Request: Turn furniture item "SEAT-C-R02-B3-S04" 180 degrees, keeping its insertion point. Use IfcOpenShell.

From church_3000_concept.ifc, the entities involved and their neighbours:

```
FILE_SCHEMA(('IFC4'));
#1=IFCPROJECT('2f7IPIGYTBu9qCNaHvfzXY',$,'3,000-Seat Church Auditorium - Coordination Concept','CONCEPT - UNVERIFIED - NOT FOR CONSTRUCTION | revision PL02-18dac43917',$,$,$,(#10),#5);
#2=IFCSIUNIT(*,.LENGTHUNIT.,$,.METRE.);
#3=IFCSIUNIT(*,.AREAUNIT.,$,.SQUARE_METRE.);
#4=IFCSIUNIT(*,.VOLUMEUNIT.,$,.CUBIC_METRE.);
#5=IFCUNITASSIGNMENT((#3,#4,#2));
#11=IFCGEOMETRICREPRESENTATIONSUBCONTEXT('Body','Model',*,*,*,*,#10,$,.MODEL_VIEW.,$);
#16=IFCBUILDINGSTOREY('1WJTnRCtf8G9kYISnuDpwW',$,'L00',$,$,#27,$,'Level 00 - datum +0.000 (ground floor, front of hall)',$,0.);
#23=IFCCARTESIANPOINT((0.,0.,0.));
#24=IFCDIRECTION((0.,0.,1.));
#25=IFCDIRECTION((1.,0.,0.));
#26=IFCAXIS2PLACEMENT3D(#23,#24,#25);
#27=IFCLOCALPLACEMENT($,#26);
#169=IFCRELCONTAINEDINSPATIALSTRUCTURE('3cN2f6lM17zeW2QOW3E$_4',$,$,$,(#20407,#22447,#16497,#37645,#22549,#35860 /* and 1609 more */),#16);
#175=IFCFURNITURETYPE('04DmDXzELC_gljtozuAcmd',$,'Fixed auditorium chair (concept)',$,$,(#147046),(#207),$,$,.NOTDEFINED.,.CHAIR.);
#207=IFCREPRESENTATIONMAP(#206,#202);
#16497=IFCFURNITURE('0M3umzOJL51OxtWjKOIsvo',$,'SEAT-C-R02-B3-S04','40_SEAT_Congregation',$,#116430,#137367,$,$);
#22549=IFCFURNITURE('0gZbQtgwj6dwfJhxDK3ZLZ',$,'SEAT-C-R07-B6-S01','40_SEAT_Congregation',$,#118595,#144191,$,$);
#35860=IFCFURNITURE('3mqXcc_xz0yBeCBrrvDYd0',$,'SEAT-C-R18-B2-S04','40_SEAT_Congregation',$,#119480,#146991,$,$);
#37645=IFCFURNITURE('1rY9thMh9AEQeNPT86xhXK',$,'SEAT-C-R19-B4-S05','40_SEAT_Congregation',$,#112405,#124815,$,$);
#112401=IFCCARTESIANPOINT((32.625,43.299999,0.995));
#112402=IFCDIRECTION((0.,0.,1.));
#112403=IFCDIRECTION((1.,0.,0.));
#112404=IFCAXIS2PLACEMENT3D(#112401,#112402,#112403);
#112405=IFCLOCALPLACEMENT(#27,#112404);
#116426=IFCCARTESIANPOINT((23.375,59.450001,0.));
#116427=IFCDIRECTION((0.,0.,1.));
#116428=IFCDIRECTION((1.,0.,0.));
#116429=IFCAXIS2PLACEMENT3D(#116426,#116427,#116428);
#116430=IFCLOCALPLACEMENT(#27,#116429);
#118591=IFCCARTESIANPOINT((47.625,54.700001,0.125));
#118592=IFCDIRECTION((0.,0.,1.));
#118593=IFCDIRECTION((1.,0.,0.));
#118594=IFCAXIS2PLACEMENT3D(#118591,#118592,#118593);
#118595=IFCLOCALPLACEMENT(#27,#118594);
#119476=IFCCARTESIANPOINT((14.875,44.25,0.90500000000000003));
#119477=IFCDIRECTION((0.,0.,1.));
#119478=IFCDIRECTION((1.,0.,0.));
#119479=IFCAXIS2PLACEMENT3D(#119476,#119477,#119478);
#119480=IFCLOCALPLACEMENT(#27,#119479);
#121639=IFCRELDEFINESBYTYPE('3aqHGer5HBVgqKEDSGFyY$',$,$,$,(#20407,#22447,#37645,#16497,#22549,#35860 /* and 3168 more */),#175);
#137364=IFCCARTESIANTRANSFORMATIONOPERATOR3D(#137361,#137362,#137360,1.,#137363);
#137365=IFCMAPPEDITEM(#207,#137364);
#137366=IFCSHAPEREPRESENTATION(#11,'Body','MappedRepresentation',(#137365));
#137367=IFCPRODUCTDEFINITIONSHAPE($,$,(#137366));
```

```python
import ifcopenshell
import ifcopenshell.api.geometry
import ifcopenshell.util.placement

model = ifcopenshell.open("church_3000_concept.ifc")

item = model.by_id(16497)
matrix = ifcopenshell.util.placement.get_local_placement(item.ObjectPlacement)
matrix = matrix @ ifcopenshell.util.placement.rotation(180, "Z")
ifcopenshell.api.geometry.edit_object_placement(model, product=item, matrix=matrix, is_si=False)

print(ifcopenshell.util.placement.get_local_placement(item.ObjectPlacement).round(3) + 0.0)

model.write("church_3000_concept-out.ifc")
```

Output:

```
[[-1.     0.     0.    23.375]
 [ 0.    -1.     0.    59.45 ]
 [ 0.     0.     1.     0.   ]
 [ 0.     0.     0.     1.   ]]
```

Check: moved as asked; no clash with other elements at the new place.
